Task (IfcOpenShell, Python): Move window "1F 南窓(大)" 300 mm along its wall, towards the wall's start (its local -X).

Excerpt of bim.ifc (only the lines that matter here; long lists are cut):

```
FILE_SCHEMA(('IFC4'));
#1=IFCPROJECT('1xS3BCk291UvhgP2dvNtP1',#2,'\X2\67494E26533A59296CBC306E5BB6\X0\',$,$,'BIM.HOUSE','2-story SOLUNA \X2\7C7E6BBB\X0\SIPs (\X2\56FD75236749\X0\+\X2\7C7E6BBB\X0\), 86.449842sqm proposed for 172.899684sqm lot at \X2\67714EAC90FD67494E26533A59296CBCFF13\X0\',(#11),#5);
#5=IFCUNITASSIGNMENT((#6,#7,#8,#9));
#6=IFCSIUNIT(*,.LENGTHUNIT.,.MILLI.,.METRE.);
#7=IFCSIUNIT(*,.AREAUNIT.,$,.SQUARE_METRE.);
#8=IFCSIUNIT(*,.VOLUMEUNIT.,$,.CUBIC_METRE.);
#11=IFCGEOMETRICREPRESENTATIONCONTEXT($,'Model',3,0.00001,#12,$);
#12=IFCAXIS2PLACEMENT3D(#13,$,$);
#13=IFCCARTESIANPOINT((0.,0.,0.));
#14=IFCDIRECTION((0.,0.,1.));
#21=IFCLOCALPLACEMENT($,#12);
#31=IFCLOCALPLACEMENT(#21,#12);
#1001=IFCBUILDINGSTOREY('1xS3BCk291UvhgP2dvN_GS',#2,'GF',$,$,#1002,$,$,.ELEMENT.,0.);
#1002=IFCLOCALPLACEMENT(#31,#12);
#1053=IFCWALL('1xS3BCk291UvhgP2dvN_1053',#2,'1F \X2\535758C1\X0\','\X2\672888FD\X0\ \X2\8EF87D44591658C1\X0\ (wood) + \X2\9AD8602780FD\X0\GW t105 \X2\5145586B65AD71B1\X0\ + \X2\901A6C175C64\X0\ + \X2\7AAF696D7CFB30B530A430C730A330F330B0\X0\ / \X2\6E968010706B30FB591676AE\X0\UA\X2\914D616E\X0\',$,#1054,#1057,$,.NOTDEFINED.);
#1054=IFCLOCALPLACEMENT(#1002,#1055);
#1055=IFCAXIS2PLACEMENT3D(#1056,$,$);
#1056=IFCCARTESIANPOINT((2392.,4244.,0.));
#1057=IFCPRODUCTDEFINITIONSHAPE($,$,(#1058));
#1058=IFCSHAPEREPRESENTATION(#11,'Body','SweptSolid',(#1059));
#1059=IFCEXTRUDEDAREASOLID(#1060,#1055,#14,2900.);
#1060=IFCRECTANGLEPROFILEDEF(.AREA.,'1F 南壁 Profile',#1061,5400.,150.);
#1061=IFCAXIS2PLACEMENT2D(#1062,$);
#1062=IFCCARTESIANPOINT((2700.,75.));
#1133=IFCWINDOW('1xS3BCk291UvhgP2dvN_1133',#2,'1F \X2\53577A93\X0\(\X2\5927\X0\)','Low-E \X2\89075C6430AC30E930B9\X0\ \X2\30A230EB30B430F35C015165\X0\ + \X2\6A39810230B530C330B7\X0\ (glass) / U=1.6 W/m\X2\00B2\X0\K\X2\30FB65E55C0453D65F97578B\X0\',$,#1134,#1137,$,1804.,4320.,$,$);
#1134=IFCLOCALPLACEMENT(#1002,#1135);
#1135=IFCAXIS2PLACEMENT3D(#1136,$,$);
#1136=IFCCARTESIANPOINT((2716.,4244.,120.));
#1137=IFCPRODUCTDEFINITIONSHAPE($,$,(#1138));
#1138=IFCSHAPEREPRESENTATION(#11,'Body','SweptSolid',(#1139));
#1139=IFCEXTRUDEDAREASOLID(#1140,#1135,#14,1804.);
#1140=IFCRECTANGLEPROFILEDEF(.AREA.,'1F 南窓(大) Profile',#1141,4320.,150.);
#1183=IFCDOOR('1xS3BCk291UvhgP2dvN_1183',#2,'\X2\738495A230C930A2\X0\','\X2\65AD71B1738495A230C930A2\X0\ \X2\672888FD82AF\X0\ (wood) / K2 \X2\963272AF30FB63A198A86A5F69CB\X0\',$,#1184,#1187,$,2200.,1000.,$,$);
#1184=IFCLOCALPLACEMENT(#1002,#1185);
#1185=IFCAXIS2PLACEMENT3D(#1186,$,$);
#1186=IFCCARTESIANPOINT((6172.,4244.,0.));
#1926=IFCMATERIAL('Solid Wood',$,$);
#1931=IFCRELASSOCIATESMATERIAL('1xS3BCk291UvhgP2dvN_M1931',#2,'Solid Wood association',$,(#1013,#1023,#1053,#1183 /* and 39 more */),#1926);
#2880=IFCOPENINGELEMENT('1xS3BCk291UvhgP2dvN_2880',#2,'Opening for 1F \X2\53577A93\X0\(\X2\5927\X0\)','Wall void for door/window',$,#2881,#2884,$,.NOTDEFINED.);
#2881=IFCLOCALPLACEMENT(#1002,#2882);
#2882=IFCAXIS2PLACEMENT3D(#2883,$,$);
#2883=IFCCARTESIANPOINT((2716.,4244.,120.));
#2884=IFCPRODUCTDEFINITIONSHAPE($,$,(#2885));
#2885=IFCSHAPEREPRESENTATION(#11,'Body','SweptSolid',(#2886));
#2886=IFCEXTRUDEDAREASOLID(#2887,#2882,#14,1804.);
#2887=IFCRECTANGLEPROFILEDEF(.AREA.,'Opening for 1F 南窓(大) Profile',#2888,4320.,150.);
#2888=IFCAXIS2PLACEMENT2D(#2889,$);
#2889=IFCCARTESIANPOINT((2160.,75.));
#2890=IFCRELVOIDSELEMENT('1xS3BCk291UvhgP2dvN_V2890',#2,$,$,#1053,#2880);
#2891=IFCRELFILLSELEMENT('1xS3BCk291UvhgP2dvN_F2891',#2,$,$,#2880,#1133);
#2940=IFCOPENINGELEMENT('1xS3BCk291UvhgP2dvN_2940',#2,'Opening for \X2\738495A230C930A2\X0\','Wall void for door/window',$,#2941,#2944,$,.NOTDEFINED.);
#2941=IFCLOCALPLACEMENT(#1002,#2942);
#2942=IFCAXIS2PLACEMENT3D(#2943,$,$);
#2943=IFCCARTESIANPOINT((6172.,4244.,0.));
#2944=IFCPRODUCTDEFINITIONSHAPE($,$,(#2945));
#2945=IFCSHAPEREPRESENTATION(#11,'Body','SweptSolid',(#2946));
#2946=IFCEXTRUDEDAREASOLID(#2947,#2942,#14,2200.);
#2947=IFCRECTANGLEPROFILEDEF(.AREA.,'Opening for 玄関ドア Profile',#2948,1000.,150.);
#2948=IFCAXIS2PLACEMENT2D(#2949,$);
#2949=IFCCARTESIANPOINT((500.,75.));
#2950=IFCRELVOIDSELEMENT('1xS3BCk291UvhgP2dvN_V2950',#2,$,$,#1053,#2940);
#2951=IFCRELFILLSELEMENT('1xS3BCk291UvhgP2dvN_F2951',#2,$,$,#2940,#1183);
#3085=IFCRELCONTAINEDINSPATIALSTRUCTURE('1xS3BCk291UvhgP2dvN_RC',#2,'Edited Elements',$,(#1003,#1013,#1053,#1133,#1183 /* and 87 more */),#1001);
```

```python
import ifcopenshell
import ifcopenshell.api.geometry
import ifcopenshell.util.placement
import ifcopenshell.util.unit

model = ifcopenshell.open("bim.ifc")
unit_scale = ifcopenshell.util.unit.calculate_unit_scale(model)

window = model.by_guid("1xS3BCk291UvhgP2dvN_1133")
opening = window.FillsVoids[0].RelatingOpeningElement
wall = opening.VoidsElements[0].RelatingBuildingElement

wall_matrix = ifcopenshell.util.placement.get_local_placement(wall.ObjectPlacement)
shift = wall_matrix[:3, 0] * -0.3 / unit_scale
before = ifcopenshell.util.placement.get_local_placement(window.ObjectPlacement)[:3, 3].copy()

# The window is not placed relative to its opening, so move both.
for product in (opening, window):
    matrix = ifcopenshell.util.placement.get_local_placement(product.ObjectPlacement)
    matrix[:3, 3] += shift
    ifcopenshell.api.geometry.edit_object_placement(model, product=product, matrix=matrix, is_si=False)

after = ifcopenshell.util.placement.get_local_placement(window.ObjectPlacement)[:3, 3]
print("window moved by", (after - before).round(3) + 0.0)

model.write("bim_updated.ifc")
```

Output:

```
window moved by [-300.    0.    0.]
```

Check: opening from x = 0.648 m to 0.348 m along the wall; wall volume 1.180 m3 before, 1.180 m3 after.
